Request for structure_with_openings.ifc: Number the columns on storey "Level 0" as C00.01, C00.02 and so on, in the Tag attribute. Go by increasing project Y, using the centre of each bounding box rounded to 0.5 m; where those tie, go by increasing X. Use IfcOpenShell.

First a look at what the model holds.

```python
import ifcopenshell
import ifcopenshell.util.element
import ifcopenshell.util.placement

model = ifcopenshell.open("structure_with_openings.ifc")
print(model.schema)
storey = next(s for s in model.by_type("IfcBuildingStorey") if s.Name == "Level 0")
columns = [e for e in ifcopenshell.util.element.get_decomposition(storey) if e.is_a("IfcColumn")]
for e in sorted(columns, key=lambda e: e.id()):
    origin = ifcopenshell.util.placement.get_local_placement(e.ObjectPlacement)[:3, 3]
    print(e.id(), e.Tag, e.Name, origin.round(2) + 0.0, sep=" | ")
```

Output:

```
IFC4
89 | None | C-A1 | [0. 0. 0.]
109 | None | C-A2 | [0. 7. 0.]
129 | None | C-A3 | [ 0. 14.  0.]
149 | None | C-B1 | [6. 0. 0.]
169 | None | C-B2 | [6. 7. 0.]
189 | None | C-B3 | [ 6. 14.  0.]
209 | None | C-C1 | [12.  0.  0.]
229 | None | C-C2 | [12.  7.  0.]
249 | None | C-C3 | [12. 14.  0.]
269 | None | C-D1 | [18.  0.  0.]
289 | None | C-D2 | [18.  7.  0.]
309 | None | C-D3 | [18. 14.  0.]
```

```python
import ifcopenshell
import ifcopenshell.geom
import ifcopenshell.util.element
import ifcopenshell.util.shape

model = ifcopenshell.open("structure_with_openings.ifc")
settings = ifcopenshell.geom.settings()
settings.set("use-world-coords", True)


def centre(element):
    shape = ifcopenshell.geom.create_shape(settings, element)
    return ifcopenshell.util.shape.get_bbox_centroid(shape.geometry)


storey = next(s for s in model.by_type("IfcBuildingStorey") if s.Name == "Level 0")
columns = [e for e in ifcopenshell.util.element.get_decomposition(storey) if e.is_a("IfcColumn")]

# Insertion points can sit at a corner or the storey origin, so sort by the geometry (in metres).
centres = {e: centre(e) for e in columns}
columns.sort(key=lambda e: (round(centres[e][1] / 0.5), centres[e][0]))

for i, e in enumerate(columns, start=1):
    number = f"C00.{i:02d}"
    e.Tag = number
    print(e.id(), number)

model.write("structure_with_openings_v2.ifc")
```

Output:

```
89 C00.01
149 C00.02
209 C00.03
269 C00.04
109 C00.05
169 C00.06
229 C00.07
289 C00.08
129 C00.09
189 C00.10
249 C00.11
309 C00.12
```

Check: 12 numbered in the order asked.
